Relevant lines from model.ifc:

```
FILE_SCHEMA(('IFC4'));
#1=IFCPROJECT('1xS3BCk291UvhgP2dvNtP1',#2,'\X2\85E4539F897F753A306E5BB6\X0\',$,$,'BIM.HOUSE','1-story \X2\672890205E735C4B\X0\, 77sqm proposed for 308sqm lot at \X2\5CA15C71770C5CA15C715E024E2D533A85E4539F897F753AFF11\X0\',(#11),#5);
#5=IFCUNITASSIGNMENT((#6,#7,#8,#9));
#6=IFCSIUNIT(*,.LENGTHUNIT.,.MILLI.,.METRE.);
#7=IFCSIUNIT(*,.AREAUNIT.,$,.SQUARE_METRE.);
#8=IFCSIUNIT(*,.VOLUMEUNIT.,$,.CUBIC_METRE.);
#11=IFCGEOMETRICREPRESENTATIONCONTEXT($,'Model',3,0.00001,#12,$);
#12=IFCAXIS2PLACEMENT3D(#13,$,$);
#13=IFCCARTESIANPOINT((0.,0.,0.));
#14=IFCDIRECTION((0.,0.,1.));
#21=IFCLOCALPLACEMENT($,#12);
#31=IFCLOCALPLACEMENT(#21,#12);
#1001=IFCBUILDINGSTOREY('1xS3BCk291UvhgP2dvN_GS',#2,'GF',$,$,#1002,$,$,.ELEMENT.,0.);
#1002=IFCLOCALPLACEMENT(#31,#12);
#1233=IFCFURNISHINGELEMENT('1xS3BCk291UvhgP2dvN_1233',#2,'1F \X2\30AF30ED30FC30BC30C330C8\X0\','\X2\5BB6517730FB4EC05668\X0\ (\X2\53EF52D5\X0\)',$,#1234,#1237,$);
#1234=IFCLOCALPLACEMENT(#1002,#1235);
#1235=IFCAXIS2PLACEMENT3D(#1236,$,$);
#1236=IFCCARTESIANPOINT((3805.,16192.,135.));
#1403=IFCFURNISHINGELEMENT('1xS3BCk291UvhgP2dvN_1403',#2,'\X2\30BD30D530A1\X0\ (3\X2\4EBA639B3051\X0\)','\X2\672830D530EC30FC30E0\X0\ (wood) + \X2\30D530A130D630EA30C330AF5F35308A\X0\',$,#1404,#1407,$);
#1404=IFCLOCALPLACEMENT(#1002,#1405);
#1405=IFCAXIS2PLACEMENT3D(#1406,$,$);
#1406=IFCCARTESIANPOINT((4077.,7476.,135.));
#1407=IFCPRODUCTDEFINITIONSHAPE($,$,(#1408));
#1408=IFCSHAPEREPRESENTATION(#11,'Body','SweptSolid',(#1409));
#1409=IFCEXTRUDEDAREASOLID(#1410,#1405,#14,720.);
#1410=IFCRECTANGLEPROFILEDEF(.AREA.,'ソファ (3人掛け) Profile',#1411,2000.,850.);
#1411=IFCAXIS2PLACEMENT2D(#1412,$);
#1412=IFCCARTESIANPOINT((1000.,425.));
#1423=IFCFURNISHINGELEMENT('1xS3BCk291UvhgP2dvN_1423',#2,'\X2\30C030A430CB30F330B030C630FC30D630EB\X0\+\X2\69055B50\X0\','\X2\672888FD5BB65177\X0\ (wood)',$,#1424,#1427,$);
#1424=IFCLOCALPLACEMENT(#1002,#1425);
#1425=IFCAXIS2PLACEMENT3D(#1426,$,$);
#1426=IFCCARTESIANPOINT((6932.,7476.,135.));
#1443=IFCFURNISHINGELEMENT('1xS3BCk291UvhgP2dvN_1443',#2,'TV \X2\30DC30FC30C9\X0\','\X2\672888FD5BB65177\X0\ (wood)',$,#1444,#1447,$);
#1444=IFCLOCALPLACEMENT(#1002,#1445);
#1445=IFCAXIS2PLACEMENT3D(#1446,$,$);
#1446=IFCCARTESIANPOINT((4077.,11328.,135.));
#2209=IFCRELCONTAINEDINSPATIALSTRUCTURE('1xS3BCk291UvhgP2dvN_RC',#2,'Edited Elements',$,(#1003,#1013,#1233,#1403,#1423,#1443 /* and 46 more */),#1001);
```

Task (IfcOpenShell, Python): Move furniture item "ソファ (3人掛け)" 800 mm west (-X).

```python
import ifcopenshell
import ifcopenshell.api.geometry
import ifcopenshell.util.placement

model = ifcopenshell.open("model.ifc")

item = model.by_guid("1xS3BCk291UvhgP2dvN_1403")
matrix = ifcopenshell.util.placement.get_local_placement(item.ObjectPlacement)
matrix[0, 3] -= 800.0
ifcopenshell.api.geometry.edit_object_placement(model, product=item, matrix=matrix, is_si=False)

print(ifcopenshell.util.placement.get_local_placement(item.ObjectPlacement).round(3) + 0.0)

model.write("model_v2.ifc")
```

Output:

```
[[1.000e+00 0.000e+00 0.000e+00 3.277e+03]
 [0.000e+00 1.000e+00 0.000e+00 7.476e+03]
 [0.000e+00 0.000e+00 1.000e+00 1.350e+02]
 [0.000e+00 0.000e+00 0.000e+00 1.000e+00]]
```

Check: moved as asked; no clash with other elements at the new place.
